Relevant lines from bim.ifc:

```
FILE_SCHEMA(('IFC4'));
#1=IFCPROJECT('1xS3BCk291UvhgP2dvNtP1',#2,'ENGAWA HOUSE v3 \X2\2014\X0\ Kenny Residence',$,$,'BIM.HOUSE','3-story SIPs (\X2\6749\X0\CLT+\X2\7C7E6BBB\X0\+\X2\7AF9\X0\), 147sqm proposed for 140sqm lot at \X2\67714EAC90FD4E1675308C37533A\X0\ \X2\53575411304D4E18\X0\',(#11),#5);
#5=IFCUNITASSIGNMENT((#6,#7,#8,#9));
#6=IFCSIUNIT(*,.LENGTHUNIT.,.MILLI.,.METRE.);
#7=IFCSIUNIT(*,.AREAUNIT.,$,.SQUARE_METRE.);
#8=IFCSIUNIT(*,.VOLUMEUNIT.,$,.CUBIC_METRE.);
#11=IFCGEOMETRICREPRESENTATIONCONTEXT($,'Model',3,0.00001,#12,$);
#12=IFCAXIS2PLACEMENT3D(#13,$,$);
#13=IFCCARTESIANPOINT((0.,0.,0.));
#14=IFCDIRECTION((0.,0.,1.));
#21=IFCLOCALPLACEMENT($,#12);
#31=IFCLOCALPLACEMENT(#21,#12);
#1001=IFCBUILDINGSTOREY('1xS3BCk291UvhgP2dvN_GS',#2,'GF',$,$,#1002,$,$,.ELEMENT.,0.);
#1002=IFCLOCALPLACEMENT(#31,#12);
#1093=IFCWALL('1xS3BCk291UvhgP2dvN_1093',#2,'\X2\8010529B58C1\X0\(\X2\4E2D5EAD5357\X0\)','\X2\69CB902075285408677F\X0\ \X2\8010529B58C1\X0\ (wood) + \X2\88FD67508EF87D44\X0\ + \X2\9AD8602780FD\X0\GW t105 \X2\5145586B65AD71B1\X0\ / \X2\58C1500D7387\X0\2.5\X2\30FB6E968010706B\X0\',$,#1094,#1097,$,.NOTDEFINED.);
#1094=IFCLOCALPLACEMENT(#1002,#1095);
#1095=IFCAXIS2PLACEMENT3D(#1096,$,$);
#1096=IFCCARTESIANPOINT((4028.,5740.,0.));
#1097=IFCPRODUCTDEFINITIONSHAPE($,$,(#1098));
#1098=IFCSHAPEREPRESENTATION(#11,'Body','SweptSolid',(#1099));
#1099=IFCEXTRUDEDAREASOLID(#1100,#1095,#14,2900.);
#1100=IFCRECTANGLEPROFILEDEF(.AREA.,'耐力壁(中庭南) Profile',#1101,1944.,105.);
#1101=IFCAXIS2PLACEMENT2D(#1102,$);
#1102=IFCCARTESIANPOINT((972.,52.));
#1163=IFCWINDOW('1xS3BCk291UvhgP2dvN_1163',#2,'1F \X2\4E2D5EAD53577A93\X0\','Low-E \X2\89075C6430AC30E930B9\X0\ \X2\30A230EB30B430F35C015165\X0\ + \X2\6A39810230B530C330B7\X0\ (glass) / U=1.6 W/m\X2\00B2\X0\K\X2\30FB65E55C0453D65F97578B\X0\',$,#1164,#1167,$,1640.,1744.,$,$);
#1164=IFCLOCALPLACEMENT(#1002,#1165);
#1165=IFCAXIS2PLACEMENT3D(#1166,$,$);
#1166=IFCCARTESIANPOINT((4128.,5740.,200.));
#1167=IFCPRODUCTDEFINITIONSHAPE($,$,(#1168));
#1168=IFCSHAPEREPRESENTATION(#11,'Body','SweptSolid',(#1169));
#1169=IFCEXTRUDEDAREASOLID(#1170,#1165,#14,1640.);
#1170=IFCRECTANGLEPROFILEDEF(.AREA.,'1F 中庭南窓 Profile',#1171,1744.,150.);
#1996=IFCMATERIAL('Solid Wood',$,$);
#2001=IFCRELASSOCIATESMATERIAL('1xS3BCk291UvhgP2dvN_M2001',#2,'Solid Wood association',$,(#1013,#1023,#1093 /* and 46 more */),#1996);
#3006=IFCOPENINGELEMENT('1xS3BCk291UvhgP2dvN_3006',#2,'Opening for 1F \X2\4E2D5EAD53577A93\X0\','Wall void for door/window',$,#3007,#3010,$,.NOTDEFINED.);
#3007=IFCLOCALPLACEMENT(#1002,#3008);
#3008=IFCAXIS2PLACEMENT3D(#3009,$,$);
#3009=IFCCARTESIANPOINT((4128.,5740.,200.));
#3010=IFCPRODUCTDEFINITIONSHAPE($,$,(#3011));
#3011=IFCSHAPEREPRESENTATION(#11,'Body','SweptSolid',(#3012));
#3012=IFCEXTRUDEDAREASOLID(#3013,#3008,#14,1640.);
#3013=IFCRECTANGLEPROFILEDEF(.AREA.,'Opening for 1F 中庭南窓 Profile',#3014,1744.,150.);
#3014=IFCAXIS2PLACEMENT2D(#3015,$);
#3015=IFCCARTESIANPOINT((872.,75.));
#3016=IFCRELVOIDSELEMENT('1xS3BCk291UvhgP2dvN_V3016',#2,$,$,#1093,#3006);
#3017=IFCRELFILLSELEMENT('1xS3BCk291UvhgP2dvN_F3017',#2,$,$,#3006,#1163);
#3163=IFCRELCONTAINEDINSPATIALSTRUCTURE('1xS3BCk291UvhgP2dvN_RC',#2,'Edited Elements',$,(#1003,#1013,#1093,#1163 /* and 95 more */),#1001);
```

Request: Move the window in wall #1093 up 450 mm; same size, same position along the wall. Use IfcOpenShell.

```python
import numpy as np
import ifcopenshell
import ifcopenshell.api.geometry
import ifcopenshell.util.placement
import ifcopenshell.util.unit

model = ifcopenshell.open("bim.ifc")
unit_scale = ifcopenshell.util.unit.calculate_unit_scale(model)

window = model.by_guid("1xS3BCk291UvhgP2dvN_1163")
opening = window.FillsVoids[0].RelatingOpeningElement
dz = 0.45 / unit_scale

shift = np.array([0.0, 0.0, dz])
# The window is not placed relative to its opening, so move both.
for product in (opening, window):
    matrix = ifcopenshell.util.placement.get_local_placement(product.ObjectPlacement)
    matrix[:3, 3] += shift
    ifcopenshell.api.geometry.edit_object_placement(model, product=product, matrix=matrix, is_si=False)

print(f"moved by {dz * unit_scale:+.3f} m")

model.write("bim-out.ifc")
```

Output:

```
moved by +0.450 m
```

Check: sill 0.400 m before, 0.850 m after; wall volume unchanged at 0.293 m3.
